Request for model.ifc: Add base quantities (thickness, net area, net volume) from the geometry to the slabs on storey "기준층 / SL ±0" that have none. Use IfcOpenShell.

First a look at what the model holds.

```python
import ifcopenshell
import ifcopenshell.util.element
import ifcopenshell.util.unit

model = ifcopenshell.open("model.ifc")
print(model.schema)
for unit_type in ("LENGTHUNIT", "AREAUNIT", "VOLUMEUNIT"):
    print(unit_type, ifcopenshell.util.unit.calculate_unit_scale(model, unit_type))
storey = next(s for s in model.by_type("IfcBuildingStorey") if s.Name == "기준층 / SL ±0")
slabs = [e for e in ifcopenshell.util.element.get_decomposition(storey) if e.is_a("IfcSlab")]
for e in sorted(slabs, key=lambda e: e.id()):
    print(e.id(), e.is_a(), e.Name, list(ifcopenshell.util.element.get_psets(e, qtos_only=True)), sep=" | ")
```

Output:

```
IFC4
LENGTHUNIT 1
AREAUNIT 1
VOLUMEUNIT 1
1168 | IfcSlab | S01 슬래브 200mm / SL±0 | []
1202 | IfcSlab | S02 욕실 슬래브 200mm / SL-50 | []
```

```python
import ifcopenshell
import ifcopenshell.api.pset
import ifcopenshell.geom
import ifcopenshell.util.element
import ifcopenshell.util.shape
import ifcopenshell.util.unit

model = ifcopenshell.open("model.ifc")
unit_scale = ifcopenshell.util.unit.calculate_unit_scale(model)
area_scale = ifcopenshell.util.unit.calculate_unit_scale(model, "AREAUNIT")
volume_scale = ifcopenshell.util.unit.calculate_unit_scale(model, "VOLUMEUNIT")
settings = ifcopenshell.geom.settings()

storey = next(s for s in model.by_type("IfcBuildingStorey") if s.Name == "기준층 / SL ±0")
slabs = [e for e in ifcopenshell.util.element.get_decomposition(storey) if e.is_a("IfcSlab")]

for e in sorted(slabs, key=lambda e: e.id()):
    if ifcopenshell.util.element.get_psets(e, qtos_only=True, should_inherit=False):
        continue
    # Geometry comes back in metres, in the element's own axes.
    shape = ifcopenshell.geom.create_shape(settings, e)
    values = {
        "Width": ifcopenshell.util.shape.get_z(shape.geometry) / unit_scale,
        "NetArea": ifcopenshell.util.shape.get_footprint_area(shape.geometry) / area_scale,
        "NetVolume": ifcopenshell.util.shape.get_volume(shape.geometry) / volume_scale,
    }
    qto = ifcopenshell.api.pset.add_qto(model, product=e, name="Qto_SlabBaseQuantities")
    ifcopenshell.api.pset.edit_qto(model, qto=qto, properties=values)
    print(e.id(), {k: round(v, 3) for k, v in values.items()})

model.write("model-out.ifc")
```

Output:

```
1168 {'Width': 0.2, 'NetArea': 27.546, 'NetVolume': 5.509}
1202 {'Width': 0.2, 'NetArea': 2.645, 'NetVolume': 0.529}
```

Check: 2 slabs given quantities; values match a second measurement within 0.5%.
